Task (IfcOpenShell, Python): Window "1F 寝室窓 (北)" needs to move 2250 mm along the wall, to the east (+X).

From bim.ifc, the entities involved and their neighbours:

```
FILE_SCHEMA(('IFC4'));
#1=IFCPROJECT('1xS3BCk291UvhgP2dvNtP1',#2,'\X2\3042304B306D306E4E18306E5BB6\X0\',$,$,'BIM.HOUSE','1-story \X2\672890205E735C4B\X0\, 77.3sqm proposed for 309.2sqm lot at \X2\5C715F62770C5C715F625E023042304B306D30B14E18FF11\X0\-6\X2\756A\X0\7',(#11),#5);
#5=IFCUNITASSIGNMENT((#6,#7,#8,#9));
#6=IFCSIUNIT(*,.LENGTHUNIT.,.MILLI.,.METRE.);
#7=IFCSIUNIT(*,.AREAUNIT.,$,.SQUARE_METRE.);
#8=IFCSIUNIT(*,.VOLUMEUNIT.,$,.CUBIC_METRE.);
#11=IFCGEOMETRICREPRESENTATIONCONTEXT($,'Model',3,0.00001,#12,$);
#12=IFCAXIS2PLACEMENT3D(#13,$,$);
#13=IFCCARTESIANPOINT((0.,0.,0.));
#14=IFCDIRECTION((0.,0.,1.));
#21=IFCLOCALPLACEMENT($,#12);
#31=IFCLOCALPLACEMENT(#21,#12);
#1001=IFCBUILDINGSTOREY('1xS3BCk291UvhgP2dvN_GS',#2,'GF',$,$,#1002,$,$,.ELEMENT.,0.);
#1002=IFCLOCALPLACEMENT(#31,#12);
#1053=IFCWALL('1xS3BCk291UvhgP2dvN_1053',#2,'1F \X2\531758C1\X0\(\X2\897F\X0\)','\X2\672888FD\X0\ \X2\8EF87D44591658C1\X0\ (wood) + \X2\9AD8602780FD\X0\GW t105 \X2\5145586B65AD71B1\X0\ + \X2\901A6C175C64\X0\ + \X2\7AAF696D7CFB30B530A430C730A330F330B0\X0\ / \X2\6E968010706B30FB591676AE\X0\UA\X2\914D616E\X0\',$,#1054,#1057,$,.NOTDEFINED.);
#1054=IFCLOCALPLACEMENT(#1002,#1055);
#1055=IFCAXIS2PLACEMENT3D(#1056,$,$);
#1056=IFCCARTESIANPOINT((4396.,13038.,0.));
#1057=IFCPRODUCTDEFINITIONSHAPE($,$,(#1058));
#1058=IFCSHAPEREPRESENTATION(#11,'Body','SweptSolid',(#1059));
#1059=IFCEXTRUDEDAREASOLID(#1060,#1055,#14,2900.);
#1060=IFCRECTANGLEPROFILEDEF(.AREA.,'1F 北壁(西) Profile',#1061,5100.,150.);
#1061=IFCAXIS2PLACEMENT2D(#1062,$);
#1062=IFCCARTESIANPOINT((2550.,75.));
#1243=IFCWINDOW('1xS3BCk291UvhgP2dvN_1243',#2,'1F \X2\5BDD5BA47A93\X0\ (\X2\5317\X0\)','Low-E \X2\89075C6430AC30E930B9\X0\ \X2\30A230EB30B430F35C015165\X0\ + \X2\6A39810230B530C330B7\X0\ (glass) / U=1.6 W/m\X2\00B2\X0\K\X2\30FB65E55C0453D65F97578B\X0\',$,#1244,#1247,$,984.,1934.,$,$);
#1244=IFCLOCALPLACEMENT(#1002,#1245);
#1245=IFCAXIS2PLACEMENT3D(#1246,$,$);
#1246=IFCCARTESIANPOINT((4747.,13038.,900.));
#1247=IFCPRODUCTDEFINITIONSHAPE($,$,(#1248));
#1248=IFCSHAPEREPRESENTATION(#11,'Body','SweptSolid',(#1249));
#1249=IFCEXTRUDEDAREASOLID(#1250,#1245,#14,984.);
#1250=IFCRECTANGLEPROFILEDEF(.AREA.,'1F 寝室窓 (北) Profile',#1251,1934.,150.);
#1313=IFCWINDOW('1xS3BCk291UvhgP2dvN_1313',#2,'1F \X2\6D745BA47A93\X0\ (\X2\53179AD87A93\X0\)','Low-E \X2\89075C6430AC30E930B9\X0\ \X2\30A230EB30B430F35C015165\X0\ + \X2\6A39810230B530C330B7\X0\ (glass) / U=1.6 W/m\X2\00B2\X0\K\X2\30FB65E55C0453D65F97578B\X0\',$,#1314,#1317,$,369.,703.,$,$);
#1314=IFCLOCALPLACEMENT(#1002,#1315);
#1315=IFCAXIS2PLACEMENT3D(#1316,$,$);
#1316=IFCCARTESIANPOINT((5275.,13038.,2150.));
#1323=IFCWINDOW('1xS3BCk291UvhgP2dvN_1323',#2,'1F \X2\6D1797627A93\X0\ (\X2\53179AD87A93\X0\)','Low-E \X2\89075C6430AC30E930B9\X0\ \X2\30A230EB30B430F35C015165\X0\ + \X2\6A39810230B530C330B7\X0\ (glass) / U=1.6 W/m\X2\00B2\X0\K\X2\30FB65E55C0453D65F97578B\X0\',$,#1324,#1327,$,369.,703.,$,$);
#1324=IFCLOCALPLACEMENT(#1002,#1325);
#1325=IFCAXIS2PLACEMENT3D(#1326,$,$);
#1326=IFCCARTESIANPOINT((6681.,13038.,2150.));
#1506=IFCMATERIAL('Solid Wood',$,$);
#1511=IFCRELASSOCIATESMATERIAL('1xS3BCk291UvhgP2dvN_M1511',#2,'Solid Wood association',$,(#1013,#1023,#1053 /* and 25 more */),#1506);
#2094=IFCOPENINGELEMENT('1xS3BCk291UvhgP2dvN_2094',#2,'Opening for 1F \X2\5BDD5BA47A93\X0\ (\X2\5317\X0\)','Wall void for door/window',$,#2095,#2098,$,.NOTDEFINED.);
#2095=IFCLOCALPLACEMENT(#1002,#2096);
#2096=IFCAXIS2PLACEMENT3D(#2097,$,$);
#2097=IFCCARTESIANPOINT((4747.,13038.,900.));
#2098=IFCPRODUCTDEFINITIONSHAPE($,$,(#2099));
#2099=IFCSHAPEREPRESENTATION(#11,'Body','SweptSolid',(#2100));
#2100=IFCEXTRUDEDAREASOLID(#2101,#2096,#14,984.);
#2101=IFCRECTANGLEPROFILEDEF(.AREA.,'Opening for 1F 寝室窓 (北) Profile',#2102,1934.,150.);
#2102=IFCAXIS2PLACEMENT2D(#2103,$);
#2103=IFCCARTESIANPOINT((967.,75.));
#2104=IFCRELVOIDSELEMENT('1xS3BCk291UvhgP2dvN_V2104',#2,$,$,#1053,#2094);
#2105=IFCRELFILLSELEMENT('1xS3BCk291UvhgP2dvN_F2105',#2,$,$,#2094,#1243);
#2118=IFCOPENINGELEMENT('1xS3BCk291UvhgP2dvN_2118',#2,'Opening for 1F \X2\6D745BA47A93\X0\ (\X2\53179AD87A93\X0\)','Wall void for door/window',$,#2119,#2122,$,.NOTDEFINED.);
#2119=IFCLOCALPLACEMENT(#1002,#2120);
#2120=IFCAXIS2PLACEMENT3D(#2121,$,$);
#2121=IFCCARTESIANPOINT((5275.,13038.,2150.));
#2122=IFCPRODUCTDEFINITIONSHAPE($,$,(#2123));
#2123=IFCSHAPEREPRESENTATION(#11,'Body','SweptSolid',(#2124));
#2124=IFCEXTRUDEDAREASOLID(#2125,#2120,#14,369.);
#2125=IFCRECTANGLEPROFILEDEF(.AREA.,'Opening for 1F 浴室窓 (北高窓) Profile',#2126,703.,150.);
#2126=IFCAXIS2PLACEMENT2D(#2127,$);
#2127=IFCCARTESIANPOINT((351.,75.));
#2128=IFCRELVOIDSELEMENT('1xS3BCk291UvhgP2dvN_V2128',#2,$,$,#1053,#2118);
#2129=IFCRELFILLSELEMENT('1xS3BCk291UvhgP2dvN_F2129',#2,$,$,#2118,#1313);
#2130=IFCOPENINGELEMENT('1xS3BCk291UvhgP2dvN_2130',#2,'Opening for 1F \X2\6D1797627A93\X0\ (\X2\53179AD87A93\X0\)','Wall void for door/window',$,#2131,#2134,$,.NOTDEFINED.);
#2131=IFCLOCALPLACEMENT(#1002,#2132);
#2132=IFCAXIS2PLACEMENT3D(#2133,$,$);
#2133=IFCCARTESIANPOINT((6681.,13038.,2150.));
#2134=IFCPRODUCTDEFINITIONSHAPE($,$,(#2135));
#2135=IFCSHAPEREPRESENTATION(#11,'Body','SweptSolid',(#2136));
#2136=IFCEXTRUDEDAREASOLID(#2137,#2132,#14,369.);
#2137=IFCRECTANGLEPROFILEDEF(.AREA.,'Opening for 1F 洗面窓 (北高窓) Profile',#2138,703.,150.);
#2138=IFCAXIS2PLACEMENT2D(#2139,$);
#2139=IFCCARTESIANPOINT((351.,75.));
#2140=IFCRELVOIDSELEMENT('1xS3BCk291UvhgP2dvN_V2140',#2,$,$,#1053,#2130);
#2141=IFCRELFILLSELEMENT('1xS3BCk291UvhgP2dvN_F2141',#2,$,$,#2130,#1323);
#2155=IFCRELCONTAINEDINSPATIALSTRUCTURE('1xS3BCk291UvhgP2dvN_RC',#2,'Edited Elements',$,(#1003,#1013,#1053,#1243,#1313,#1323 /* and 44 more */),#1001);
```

```python
import ifcopenshell
import ifcopenshell.api.geometry
import ifcopenshell.util.placement
import ifcopenshell.util.unit

model = ifcopenshell.open("bim.ifc")
unit_scale = ifcopenshell.util.unit.calculate_unit_scale(model)

window = model.by_id(1243)
opening = window.FillsVoids[0].RelatingOpeningElement
wall = opening.VoidsElements[0].RelatingBuildingElement

wall_matrix = ifcopenshell.util.placement.get_local_placement(wall.ObjectPlacement)
shift = wall_matrix[:3, 0] * 2.25 / unit_scale
before = ifcopenshell.util.placement.get_local_placement(window.ObjectPlacement)[:3, 3].copy()

# The window is not placed relative to its opening, so move both.
for product in (opening, window):
    matrix = ifcopenshell.util.placement.get_local_placement(product.ObjectPlacement)
    matrix[:3, 3] += shift
    ifcopenshell.api.geometry.edit_object_placement(model, product=product, matrix=matrix, is_si=False)

after = ifcopenshell.util.placement.get_local_placement(window.ObjectPlacement)[:3, 3]
print("window moved by", (after - before).round(3) + 0.0)

model.write("bim_v2.ifc")
```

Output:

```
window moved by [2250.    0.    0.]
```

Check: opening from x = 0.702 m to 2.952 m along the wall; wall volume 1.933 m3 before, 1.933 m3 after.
